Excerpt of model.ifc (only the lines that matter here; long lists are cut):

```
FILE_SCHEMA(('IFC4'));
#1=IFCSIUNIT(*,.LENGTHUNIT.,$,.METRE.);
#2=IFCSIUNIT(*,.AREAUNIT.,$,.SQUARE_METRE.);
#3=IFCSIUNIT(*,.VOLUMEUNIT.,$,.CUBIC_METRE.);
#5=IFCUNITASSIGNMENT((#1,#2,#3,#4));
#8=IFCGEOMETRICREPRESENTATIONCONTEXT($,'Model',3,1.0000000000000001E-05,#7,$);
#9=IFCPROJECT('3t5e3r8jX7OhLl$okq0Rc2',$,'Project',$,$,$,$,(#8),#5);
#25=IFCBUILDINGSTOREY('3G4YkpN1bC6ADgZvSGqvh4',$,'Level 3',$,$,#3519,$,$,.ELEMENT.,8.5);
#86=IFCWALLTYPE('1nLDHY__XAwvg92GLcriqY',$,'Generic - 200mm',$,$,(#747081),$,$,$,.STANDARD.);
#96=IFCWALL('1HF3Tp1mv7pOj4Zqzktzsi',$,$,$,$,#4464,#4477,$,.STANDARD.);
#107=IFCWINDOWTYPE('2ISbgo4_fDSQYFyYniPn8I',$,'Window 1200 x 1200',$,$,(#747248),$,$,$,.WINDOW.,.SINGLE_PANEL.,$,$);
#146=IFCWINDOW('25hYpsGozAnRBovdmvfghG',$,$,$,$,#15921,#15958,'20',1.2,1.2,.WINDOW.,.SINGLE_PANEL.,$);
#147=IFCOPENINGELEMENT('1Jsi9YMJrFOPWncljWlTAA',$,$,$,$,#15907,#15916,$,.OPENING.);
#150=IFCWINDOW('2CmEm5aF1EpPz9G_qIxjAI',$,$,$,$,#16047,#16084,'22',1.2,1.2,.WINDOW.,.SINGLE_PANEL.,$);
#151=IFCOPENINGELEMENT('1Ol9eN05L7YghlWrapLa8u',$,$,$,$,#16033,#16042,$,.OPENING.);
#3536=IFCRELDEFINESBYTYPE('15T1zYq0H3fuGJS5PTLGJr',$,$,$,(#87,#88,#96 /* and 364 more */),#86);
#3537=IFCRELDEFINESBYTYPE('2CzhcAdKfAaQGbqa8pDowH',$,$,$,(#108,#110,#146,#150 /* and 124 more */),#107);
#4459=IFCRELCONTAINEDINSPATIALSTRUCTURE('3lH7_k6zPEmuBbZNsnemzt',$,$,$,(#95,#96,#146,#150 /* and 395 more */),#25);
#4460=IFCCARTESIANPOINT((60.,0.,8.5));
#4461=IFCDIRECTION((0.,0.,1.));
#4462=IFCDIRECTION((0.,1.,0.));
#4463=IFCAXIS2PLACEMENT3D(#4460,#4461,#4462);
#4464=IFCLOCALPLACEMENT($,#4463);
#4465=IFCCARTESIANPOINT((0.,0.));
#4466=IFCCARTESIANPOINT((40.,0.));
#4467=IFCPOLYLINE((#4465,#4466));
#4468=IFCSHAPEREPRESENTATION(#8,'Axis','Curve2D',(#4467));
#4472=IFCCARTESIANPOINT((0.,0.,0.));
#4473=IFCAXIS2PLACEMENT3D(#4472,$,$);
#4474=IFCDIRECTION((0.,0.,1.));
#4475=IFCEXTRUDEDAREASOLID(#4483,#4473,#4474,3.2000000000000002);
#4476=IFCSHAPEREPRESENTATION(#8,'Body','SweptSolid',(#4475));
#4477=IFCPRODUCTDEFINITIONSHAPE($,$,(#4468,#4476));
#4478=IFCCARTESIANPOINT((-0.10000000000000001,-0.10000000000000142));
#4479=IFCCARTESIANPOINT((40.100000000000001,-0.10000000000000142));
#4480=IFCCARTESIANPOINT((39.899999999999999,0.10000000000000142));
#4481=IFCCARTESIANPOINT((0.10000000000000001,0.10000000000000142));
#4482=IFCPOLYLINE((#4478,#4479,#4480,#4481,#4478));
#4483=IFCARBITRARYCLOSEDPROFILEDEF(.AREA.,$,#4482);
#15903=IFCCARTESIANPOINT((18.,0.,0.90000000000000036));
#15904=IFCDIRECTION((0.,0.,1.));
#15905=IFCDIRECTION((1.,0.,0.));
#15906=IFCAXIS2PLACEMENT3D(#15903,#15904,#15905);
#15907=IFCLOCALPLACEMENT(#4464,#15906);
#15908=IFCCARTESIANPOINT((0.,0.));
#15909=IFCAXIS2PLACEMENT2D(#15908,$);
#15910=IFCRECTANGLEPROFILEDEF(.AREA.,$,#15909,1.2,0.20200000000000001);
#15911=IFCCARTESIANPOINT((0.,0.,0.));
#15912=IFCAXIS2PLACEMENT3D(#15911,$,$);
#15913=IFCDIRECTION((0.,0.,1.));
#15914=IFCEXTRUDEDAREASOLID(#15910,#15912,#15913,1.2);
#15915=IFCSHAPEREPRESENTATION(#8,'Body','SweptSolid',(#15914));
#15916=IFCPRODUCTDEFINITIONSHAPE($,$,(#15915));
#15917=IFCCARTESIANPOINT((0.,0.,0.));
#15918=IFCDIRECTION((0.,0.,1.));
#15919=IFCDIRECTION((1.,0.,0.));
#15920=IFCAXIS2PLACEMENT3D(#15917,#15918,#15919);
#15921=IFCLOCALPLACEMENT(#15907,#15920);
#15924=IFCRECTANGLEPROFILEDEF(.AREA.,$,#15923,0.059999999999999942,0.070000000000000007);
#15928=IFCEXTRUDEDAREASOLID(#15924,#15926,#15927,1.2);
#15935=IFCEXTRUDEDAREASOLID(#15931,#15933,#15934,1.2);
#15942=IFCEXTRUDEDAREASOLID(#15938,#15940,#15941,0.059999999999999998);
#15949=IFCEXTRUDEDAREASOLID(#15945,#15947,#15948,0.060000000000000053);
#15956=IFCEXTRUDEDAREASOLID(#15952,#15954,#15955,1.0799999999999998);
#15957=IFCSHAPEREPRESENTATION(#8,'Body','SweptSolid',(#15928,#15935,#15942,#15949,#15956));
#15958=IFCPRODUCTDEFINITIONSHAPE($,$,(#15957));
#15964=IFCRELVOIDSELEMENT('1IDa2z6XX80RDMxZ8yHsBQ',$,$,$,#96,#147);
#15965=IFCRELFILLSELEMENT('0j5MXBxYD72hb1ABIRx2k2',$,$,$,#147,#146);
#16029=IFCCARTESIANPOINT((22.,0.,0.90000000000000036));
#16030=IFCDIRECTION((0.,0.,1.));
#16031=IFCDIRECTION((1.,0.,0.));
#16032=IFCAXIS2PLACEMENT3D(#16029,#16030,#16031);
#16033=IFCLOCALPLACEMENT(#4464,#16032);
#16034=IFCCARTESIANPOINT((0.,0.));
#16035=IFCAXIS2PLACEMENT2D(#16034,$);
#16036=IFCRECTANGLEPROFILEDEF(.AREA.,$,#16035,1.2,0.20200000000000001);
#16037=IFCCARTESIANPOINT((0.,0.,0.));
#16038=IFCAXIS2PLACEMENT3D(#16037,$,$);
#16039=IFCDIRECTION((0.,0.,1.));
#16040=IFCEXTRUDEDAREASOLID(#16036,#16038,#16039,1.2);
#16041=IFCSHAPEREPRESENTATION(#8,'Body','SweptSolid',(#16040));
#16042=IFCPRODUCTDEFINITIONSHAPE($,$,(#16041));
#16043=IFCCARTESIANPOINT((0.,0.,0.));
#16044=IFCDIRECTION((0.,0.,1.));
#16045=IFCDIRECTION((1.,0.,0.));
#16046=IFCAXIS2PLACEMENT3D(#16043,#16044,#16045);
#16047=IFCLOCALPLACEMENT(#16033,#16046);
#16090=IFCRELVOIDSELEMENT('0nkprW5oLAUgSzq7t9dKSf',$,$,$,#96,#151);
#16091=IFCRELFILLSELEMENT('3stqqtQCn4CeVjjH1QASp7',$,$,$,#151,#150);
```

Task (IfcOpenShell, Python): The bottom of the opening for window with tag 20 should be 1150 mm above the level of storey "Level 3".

```python
import numpy as np
import ifcopenshell
import ifcopenshell.api.geometry
import ifcopenshell.geom
import ifcopenshell.util.element
import ifcopenshell.util.placement
import ifcopenshell.util.shape
import ifcopenshell.util.unit

model = ifcopenshell.open("model.ifc")
unit_scale = ifcopenshell.util.unit.calculate_unit_scale(model)

window = model.by_id(146)
opening = window.FillsVoids[0].RelatingOpeningElement
storey = ifcopenshell.util.element.get_container(window, ifc_class="IfcBuildingStorey")
level = ifcopenshell.util.placement.get_local_placement(storey.ObjectPlacement)[2, 3]

# The opening's origin need not be at the sill, so measure its lowest point.
shape = ifcopenshell.geom.create_shape(ifcopenshell.geom.settings(), opening)
bottom = ifcopenshell.util.shape.get_shape_bottom_elevation(shape, shape.geometry) / unit_scale
dz = level + 1.15 / unit_scale - bottom

shift = np.array([0.0, 0.0, dz])
# The window is placed relative to its opening, so it follows when the opening moves.
matrix = ifcopenshell.util.placement.get_local_placement(opening.ObjectPlacement)
matrix[:3, 3] += shift
ifcopenshell.api.geometry.edit_object_placement(
    model, product=opening, matrix=matrix, is_si=False, should_transform_children=True
)

print(f"moved by {dz * unit_scale:+.3f} m")

model.write("model_v2.ifc")
```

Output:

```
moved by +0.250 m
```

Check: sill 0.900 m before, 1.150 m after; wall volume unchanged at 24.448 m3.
